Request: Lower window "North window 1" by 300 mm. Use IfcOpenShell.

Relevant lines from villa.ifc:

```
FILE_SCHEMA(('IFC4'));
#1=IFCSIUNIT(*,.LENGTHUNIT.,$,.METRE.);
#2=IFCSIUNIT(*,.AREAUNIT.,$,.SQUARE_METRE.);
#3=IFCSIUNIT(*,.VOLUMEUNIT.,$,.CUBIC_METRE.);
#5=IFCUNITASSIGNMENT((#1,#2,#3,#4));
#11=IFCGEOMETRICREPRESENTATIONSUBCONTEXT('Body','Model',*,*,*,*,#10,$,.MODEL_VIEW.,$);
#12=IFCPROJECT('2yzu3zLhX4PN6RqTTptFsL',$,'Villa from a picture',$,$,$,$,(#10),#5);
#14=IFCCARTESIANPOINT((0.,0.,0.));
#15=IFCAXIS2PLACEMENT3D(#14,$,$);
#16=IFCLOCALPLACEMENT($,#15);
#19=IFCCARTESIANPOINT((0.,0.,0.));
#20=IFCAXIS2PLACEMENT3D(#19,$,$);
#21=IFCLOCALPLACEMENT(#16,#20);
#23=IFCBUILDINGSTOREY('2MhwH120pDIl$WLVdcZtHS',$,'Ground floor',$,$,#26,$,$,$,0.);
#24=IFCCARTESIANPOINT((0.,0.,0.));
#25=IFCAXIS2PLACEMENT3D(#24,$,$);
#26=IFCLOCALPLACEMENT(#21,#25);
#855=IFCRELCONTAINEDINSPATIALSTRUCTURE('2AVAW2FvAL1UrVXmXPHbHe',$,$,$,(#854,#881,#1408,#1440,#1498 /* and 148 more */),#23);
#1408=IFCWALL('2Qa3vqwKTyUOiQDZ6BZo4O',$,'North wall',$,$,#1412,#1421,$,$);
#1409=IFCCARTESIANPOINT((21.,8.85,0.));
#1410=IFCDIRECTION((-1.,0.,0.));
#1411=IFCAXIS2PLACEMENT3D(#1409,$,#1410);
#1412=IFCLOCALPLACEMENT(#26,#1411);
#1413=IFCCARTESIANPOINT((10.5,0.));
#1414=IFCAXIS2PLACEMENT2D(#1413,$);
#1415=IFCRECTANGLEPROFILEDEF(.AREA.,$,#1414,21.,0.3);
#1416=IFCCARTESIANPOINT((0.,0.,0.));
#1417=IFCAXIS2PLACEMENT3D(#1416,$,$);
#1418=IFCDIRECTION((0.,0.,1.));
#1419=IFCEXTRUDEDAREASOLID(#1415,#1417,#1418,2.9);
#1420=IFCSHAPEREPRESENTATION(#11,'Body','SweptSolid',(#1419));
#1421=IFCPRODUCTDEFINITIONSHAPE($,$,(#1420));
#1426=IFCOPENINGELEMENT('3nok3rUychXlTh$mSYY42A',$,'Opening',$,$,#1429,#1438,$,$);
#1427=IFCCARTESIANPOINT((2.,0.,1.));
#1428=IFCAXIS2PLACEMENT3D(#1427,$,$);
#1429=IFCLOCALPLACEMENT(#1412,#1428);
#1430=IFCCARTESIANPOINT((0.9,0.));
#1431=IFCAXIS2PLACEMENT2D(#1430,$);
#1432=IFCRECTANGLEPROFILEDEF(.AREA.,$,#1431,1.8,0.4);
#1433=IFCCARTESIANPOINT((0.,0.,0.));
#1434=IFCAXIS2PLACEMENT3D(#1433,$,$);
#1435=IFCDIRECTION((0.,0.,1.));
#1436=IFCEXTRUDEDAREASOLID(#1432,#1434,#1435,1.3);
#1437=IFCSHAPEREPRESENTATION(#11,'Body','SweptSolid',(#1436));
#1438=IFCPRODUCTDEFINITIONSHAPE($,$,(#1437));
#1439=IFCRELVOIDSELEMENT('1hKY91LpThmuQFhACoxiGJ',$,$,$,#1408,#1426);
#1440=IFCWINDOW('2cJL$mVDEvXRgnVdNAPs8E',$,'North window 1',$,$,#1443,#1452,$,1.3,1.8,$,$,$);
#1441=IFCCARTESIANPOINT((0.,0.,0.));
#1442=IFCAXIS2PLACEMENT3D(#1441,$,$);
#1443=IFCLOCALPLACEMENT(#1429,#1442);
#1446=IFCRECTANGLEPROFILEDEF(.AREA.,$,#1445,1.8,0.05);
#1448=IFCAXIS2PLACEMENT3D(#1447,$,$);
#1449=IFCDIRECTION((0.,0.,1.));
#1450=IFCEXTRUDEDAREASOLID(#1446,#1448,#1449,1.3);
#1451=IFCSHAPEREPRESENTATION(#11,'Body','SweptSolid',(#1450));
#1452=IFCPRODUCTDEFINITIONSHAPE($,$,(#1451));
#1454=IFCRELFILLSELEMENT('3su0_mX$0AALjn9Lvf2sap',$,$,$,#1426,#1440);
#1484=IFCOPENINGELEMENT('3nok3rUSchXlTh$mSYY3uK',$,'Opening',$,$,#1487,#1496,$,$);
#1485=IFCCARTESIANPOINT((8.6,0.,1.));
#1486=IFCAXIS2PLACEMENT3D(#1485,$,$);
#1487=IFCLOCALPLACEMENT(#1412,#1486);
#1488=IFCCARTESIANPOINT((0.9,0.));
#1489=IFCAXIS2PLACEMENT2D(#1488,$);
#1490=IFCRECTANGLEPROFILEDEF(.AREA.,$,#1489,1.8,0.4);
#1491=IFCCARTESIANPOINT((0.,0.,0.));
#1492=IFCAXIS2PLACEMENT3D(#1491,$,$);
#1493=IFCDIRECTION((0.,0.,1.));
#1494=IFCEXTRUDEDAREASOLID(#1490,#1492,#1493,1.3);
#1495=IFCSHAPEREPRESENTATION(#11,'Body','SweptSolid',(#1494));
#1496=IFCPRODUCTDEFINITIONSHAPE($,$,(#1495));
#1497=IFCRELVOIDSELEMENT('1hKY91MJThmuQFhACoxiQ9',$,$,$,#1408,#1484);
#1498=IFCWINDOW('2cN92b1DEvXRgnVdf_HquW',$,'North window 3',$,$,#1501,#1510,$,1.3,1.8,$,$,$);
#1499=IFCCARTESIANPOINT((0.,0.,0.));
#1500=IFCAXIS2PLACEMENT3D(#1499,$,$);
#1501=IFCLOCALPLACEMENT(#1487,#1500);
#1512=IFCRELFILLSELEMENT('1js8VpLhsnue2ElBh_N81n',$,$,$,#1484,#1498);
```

```python
import numpy as np
import ifcopenshell
import ifcopenshell.api.geometry
import ifcopenshell.util.placement
import ifcopenshell.util.unit

model = ifcopenshell.open("villa.ifc")
unit_scale = ifcopenshell.util.unit.calculate_unit_scale(model)

window = model.by_guid("2cJL$mVDEvXRgnVdNAPs8E")
opening = window.FillsVoids[0].RelatingOpeningElement
dz = -0.3 / unit_scale

shift = np.array([0.0, 0.0, dz])
# The window is placed relative to its opening, so it follows when the opening moves.
matrix = ifcopenshell.util.placement.get_local_placement(opening.ObjectPlacement)
matrix[:3, 3] += shift
ifcopenshell.api.geometry.edit_object_placement(
    model, product=opening, matrix=matrix, is_si=False, should_transform_children=True
)

print(f"moved by {dz * unit_scale:+.3f} m")

model.write("villa_rev.ifc")
```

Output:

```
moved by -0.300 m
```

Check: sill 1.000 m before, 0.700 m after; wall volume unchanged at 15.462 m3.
